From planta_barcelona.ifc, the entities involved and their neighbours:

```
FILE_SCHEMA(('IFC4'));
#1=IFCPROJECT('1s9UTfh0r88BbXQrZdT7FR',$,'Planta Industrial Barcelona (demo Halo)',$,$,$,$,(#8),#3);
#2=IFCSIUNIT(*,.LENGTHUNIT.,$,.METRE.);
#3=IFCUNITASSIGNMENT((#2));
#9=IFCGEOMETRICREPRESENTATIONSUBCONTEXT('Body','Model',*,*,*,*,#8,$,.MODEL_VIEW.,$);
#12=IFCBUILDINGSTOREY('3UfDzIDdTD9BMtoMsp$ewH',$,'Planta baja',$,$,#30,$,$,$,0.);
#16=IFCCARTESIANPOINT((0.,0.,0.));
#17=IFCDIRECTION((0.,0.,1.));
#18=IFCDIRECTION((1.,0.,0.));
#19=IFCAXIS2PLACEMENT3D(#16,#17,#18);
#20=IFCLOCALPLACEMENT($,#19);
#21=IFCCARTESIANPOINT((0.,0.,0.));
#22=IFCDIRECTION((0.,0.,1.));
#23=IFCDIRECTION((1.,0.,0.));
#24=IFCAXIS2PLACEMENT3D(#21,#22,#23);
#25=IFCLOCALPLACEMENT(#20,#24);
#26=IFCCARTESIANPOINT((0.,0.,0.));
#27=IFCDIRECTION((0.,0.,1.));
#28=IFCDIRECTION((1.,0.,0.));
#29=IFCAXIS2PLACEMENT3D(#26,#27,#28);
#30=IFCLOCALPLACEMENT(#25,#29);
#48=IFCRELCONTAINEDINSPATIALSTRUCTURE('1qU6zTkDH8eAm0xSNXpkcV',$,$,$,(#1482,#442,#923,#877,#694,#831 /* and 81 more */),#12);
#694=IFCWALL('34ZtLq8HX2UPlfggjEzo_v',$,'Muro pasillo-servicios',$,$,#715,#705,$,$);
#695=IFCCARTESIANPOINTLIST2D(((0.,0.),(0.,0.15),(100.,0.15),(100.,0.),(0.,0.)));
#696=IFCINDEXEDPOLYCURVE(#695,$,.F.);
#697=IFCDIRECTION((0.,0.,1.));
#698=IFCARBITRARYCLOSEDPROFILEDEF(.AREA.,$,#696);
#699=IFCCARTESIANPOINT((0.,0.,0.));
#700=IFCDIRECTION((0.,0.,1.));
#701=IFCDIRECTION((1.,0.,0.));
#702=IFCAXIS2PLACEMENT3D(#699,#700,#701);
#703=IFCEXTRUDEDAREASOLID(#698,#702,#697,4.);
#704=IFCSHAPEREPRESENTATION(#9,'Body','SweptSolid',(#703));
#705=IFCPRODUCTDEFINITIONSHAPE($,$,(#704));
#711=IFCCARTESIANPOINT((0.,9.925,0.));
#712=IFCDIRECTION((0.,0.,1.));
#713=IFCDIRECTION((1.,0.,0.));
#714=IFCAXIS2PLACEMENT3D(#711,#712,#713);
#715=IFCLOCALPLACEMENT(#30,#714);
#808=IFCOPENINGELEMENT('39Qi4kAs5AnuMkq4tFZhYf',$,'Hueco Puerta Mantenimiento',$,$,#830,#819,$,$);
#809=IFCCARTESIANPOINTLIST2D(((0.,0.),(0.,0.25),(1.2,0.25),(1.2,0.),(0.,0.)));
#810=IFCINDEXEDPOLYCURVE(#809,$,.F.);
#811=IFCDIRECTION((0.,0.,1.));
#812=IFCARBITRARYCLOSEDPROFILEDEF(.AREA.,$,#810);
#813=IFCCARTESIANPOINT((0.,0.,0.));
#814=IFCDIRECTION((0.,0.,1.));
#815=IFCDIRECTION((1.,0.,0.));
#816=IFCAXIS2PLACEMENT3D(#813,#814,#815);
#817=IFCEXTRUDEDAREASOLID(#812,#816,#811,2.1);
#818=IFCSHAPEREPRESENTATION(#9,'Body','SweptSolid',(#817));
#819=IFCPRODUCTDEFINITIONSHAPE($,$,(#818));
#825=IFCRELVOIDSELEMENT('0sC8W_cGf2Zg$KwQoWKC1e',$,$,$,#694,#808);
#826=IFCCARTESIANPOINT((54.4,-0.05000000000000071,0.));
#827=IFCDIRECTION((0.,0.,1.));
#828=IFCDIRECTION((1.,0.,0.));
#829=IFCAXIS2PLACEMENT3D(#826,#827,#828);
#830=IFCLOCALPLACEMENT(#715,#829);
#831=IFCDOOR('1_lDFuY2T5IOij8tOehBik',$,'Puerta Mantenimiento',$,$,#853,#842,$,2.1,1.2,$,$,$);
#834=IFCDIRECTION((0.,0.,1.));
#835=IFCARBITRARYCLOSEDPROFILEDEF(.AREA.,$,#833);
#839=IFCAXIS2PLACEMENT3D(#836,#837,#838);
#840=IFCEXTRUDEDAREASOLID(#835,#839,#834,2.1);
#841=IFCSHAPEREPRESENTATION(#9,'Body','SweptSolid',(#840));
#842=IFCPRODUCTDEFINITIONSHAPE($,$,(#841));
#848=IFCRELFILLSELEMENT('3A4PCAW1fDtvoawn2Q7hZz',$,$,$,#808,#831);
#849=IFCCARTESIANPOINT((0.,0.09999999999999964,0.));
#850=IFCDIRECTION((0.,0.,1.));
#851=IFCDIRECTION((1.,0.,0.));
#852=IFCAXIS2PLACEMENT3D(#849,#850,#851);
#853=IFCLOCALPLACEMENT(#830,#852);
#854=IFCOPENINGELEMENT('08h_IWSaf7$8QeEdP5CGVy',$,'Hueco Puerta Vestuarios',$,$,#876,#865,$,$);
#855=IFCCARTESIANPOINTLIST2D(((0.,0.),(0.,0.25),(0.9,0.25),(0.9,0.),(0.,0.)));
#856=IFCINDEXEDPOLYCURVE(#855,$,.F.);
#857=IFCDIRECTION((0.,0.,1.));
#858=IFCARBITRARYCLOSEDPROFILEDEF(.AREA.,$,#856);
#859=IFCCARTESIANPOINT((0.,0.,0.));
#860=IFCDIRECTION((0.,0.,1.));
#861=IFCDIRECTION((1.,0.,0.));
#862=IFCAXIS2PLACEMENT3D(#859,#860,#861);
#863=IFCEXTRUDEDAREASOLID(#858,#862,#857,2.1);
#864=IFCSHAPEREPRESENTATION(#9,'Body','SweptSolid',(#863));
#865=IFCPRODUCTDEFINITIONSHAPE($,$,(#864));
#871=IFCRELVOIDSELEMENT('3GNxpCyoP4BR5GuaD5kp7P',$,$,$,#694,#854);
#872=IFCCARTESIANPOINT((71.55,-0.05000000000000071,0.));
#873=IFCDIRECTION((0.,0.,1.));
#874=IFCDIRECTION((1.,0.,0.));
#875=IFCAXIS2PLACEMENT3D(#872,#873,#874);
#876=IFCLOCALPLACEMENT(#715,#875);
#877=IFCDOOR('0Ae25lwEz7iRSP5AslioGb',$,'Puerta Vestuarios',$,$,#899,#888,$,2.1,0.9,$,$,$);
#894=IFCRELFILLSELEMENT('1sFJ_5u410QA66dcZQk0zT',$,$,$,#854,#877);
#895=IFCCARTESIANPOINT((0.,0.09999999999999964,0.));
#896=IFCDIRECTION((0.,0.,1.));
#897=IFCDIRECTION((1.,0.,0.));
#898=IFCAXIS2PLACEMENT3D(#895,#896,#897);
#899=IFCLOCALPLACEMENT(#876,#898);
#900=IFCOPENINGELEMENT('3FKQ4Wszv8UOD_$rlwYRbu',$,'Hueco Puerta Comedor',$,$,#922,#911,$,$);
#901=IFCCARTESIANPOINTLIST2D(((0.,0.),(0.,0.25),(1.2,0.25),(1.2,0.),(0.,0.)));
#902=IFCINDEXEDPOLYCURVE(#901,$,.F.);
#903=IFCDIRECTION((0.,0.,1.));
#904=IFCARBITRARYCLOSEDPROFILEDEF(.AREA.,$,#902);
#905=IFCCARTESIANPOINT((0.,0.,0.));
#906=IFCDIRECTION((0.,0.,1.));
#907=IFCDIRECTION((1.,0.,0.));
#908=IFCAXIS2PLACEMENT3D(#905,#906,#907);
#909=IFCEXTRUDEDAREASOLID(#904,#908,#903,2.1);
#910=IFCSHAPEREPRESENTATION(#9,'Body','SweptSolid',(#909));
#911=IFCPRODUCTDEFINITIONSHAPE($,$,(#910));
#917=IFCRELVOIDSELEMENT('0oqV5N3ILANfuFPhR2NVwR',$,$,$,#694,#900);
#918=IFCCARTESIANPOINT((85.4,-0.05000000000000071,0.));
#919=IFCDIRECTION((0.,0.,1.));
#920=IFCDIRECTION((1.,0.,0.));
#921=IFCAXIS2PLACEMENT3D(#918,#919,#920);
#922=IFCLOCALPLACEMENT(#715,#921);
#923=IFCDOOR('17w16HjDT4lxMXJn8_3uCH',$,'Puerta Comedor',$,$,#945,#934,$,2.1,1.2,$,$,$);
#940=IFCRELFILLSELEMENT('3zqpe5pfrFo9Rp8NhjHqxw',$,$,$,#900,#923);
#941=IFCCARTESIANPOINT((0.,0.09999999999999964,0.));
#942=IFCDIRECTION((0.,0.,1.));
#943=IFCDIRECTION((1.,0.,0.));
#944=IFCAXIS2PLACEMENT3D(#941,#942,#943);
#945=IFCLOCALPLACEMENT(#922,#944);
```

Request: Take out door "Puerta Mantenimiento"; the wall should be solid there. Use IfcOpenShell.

```python
import ifcopenshell
import ifcopenshell.api.feature
import ifcopenshell.api.root
import ifcopenshell.geom
import ifcopenshell.util.shape

model = ifcopenshell.open("planta_barcelona.ifc")
settings = ifcopenshell.geom.settings()


def volume(element):
    """Net volume in cubic metres, openings subtracted."""
    shape = ifcopenshell.geom.create_shape(settings, element)
    return ifcopenshell.util.shape.get_volume(shape.geometry)


door = model.by_id(831)
opening = door.FillsVoids[0].RelatingOpeningElement
wall = opening.VoidsElements[0].RelatingBuildingElement
before = volume(wall)

ifcopenshell.api.root.remove_product(model, product=door)
ifcopenshell.api.feature.remove_feature(model, feature=opening)

after = volume(wall)

print(f"wall volume {before:.3f} -> {after:.3f} m3")

model.write("planta_barcelona_rev.ifc")
```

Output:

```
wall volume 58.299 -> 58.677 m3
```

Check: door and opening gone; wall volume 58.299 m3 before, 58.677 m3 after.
